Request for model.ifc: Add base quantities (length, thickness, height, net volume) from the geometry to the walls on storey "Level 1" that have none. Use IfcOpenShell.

First a look at what the model holds.

```python
import ifcopenshell
import ifcopenshell.util.element
import ifcopenshell.util.unit

model = ifcopenshell.open("model.ifc")
print(model.schema)
for unit_type in ("LENGTHUNIT", "AREAUNIT", "VOLUMEUNIT"):
    print(unit_type, ifcopenshell.util.unit.calculate_unit_scale(model, unit_type))
storey = next(s for s in model.by_type("IfcBuildingStorey") if s.Name == "Level 1")
walls = [e for e in ifcopenshell.util.element.get_decomposition(storey) if e.is_a("IfcWall")]
for e in sorted(walls, key=lambda e: e.id()):
    print(e.id(), e.is_a(), e.Name, list(ifcopenshell.util.element.get_psets(e, qtos_only=True)), sep=" | ")
```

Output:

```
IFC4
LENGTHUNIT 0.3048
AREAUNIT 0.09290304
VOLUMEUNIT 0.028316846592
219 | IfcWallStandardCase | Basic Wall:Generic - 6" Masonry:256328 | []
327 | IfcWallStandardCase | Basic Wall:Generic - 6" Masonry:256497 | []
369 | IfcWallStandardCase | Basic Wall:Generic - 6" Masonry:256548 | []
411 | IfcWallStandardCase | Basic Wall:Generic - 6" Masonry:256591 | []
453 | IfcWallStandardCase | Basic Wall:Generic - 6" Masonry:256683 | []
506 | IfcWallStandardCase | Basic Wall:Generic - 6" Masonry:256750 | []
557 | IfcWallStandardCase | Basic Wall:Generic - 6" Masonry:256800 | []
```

```python
import ifcopenshell
import ifcopenshell.api.pset
import ifcopenshell.geom
import ifcopenshell.util.element
import ifcopenshell.util.shape
import ifcopenshell.util.unit

model = ifcopenshell.open("model.ifc")
unit_scale = ifcopenshell.util.unit.calculate_unit_scale(model)
volume_scale = ifcopenshell.util.unit.calculate_unit_scale(model, "VOLUMEUNIT")
settings = ifcopenshell.geom.settings()

storey = next(s for s in model.by_type("IfcBuildingStorey") if s.Name == "Level 1")
walls = [e for e in ifcopenshell.util.element.get_decomposition(storey) if e.is_a("IfcWall")]

for e in sorted(walls, key=lambda e: e.id()):
    if ifcopenshell.util.element.get_psets(e, qtos_only=True, should_inherit=False):
        continue
    # Geometry comes back in metres, in the element's own axes.
    shape = ifcopenshell.geom.create_shape(settings, e)
    values = {
        "Length": ifcopenshell.util.shape.get_x(shape.geometry) / unit_scale,
        "Width": ifcopenshell.util.shape.get_y(shape.geometry) / unit_scale,
        "Height": ifcopenshell.util.shape.get_z(shape.geometry) / unit_scale,
        "NetVolume": ifcopenshell.util.shape.get_volume(shape.geometry) / volume_scale,
    }
    qto = ifcopenshell.api.pset.add_qto(model, product=e, name="Qto_WallBaseQuantities")
    ifcopenshell.api.pset.edit_qto(model, qto=qto, properties=values)
    print(e.id(), {k: round(v, 3) for k, v in values.items()})

model.write("model_edited.ifc")
```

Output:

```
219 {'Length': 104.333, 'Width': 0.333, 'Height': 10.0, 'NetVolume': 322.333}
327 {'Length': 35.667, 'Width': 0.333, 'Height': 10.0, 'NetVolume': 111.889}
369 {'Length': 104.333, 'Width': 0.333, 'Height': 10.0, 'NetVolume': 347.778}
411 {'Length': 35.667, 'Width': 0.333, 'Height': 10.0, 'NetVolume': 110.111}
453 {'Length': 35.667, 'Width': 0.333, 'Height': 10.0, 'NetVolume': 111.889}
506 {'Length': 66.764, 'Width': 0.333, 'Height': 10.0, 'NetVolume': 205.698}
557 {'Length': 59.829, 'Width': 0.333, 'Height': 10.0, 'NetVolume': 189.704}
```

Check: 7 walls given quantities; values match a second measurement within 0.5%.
